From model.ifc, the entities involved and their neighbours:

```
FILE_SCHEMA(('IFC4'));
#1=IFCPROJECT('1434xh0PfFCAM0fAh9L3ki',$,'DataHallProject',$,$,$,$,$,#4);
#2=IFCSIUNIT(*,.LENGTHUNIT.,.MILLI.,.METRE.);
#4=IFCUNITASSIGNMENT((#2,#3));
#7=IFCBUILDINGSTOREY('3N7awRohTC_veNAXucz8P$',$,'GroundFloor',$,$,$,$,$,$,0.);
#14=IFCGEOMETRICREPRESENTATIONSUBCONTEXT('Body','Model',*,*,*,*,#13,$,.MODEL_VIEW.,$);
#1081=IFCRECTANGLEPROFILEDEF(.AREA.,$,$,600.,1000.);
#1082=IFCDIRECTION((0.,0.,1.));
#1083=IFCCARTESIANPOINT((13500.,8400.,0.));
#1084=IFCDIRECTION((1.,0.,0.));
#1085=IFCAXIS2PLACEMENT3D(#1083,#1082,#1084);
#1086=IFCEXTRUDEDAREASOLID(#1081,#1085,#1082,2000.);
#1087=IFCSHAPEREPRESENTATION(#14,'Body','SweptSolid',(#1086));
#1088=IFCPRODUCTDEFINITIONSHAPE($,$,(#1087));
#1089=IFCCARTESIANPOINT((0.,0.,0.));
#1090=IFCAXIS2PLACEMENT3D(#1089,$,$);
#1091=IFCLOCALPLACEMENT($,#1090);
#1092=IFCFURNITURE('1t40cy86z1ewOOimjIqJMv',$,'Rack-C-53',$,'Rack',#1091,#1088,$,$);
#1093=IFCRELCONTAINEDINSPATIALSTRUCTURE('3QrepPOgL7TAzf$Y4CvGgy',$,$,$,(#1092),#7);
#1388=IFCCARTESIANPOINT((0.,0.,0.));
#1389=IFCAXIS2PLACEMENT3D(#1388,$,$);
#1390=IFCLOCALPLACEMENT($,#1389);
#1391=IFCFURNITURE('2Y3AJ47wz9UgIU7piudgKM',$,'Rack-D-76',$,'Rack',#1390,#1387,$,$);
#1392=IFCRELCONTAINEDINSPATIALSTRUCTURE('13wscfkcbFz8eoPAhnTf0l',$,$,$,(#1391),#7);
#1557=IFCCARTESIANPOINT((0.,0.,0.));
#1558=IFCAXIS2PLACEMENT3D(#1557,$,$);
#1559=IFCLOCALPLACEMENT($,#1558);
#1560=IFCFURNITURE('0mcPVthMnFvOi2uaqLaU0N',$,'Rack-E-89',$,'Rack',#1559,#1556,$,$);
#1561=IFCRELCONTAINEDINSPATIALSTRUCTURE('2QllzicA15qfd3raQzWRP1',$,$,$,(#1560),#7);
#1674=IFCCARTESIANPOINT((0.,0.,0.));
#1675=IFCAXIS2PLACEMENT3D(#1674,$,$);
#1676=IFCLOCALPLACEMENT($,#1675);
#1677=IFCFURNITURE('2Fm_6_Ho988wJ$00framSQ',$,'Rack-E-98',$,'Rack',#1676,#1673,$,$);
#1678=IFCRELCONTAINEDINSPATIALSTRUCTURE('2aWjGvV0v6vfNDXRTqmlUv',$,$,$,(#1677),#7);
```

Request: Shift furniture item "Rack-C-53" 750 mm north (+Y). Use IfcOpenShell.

```python
import ifcopenshell
import ifcopenshell.api.geometry
import ifcopenshell.util.placement
import ifcopenshell.util.unit

model = ifcopenshell.open("model.ifc")
unit_scale = ifcopenshell.util.unit.calculate_unit_scale(model)

item = model.by_id(1092)
matrix = ifcopenshell.util.placement.get_local_placement(item.ObjectPlacement)
matrix[1, 3] += 0.75 / unit_scale
ifcopenshell.api.geometry.edit_object_placement(model, product=item, matrix=matrix, is_si=False)

print(ifcopenshell.util.placement.get_local_placement(item.ObjectPlacement).round(3) + 0.0)

model.write("model_rev.ifc")
```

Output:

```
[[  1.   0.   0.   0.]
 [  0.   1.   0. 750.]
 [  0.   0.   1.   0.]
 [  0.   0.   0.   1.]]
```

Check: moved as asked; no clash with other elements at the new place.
